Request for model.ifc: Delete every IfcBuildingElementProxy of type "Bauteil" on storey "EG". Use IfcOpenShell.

First a look at what the model holds.

```python
import ifcopenshell
import ifcopenshell.util.element

model = ifcopenshell.open("model.ifc")
print(model.schema)
storey = next(s for s in model.by_type("IfcBuildingStorey") if s.Name == "EG")
proxies = [e for e in ifcopenshell.util.element.get_decomposition(storey) if e.is_a("IfcBuildingElementProxy")]
seen = {}
for e in proxies:
    element_type = ifcopenshell.util.element.get_type(e)
    name = element_type.Name if element_type not in (None, e) else None
    seen[name] = seen.get(name, 0) + 1
for name, count in sorted(seen.items(), key=str):
    print(count, "x", name)
```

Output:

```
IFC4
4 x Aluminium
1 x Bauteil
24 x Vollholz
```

```python
import ifcopenshell
import ifcopenshell.api.root
import ifcopenshell.util.element

model = ifcopenshell.open("model.ifc")

storey = next(s for s in model.by_type("IfcBuildingStorey") if s.Name == "EG")
proxies = [e for e in ifcopenshell.util.element.get_decomposition(storey) if e.is_a("IfcBuildingElementProxy")]
targets = [e for e in proxies if (t := ifcopenshell.util.element.get_type(e)) not in (None, e) and t.Name == "Bauteil"]

for e in targets:
    ifcopenshell.api.root.remove_product(model, product=e)
print(len(targets), "removed")

model.write("model_v2.ifc")
```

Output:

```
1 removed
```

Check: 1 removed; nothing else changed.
